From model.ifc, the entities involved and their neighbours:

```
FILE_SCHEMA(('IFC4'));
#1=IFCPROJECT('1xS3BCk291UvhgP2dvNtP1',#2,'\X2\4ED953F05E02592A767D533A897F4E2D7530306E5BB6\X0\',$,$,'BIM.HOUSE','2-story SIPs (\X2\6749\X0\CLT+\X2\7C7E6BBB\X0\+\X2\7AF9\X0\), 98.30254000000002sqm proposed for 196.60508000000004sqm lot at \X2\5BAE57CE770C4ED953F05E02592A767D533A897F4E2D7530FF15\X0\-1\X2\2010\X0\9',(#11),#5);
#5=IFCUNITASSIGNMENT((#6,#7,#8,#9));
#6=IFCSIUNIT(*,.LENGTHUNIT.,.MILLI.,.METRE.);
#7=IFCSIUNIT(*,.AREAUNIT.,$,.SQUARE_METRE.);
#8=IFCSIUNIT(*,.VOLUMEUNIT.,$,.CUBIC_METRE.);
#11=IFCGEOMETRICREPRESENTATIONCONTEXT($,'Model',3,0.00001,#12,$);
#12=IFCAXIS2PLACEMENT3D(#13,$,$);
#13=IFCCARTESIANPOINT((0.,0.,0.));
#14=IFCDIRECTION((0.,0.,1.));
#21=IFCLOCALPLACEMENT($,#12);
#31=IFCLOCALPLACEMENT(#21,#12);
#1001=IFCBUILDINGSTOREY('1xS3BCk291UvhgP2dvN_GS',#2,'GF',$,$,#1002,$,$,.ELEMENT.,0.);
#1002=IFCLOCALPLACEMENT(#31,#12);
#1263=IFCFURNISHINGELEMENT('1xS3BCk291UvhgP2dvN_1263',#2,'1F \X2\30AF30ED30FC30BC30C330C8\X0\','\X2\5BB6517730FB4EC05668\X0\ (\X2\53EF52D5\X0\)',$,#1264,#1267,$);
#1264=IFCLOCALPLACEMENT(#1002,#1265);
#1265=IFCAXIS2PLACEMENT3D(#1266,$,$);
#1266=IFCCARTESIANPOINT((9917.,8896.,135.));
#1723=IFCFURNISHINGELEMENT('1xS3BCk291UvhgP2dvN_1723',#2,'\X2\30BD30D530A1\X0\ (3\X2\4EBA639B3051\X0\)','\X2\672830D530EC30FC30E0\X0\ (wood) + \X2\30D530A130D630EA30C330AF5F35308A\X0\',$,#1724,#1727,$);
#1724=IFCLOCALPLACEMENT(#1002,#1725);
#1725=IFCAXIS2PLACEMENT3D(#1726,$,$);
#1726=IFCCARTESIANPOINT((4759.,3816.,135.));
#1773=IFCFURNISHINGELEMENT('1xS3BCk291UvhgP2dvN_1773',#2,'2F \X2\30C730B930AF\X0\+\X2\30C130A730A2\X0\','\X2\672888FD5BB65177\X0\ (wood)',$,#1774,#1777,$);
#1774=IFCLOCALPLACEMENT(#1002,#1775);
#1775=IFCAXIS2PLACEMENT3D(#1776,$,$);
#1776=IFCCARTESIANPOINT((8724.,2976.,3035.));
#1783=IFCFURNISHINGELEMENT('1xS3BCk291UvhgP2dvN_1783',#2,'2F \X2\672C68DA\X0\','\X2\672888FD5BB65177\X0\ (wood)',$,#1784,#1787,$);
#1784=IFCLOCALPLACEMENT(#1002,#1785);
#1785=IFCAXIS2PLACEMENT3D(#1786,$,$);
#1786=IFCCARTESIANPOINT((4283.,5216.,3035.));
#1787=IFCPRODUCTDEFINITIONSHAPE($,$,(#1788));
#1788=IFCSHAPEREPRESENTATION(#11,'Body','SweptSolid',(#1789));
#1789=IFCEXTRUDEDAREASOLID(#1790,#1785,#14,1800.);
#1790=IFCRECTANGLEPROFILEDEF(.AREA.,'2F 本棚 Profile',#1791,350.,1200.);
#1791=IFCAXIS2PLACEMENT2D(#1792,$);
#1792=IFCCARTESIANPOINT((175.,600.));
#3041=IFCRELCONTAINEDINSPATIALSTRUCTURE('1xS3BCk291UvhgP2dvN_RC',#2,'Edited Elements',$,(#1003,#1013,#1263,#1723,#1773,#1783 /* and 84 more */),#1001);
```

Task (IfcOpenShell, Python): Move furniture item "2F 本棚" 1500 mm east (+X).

```python
import ifcopenshell
import ifcopenshell.api.geometry
import ifcopenshell.util.placement
import ifcopenshell.util.unit

model = ifcopenshell.open("model.ifc")
unit_scale = ifcopenshell.util.unit.calculate_unit_scale(model)

item = model.by_guid("1xS3BCk291UvhgP2dvN_1783")
matrix = ifcopenshell.util.placement.get_local_placement(item.ObjectPlacement)
matrix[0, 3] += 1.5 / unit_scale
ifcopenshell.api.geometry.edit_object_placement(model, product=item, matrix=matrix, is_si=False)

print(ifcopenshell.util.placement.get_local_placement(item.ObjectPlacement).round(3) + 0.0)

model.write("model_edited.ifc")
```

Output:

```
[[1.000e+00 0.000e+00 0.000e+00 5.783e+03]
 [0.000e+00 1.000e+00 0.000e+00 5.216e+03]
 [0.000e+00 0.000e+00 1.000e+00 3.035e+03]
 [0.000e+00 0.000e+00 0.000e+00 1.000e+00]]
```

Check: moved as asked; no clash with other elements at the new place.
